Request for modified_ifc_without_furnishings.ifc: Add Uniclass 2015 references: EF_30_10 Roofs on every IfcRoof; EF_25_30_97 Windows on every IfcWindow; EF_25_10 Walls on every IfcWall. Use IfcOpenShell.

First a look at what the model holds.

```python
import ifcopenshell

model = ifcopenshell.open("modified_ifc_without_furnishings.ifc")
print(model.schema)
print("classifications:", [c.Name for c in model.by_type("IfcClassification")])
for ifc_class in ("IfcDoor", "IfcRoof", "IfcStair", "IfcWall", "IfcWindow"):
    print(ifc_class, len(model.by_type(ifc_class)))
```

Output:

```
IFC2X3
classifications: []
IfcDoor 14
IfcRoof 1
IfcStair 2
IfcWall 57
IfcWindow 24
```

```python
import ifcopenshell
import ifcopenshell.api.classification

model = ifcopenshell.open("modified_ifc_without_furnishings.ifc")

# IFC2X3 requires Source and Edition and has no link from the project to the system.
system = model.create_entity("IfcClassification", Source="NBS", Edition="2015", Name="Uniclass 2015")

codes = {
    "IfcRoof": ("EF_30_10", "Roofs"),
    "IfcWindow": ("EF_25_30_97", "Windows"),
    "IfcWall": ("EF_25_10", "Walls"),
}
for ifc_class, (code, name) in codes.items():
    products = model.by_type(ifc_class)
    ifcopenshell.api.classification.add_reference(
        model, products=products, classification=system, identification=code, name=name
    )
    print(code, len(products))

model.write("modified_ifc_without_furnishings_rev.ifc")
```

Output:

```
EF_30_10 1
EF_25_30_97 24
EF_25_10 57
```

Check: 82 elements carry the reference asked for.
